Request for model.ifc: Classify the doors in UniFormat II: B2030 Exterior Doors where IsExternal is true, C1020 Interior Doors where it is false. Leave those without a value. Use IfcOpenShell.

First a look at what the model holds.

```python
import ifcopenshell
import ifcopenshell.util.element

model = ifcopenshell.open("model.ifc")
print(model.schema)
print("classifications:", [c.Name for c in model.by_type("IfcClassification")])
values = [ifcopenshell.util.element.get_pset(e, "Pset_DoorCommon", "IsExternal") for e in model.by_type("IfcDoor")]
for value in (True, False, None):
    print("IsExternal", value, values.count(value))
```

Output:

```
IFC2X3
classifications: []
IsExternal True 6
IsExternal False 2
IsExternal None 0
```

```python
import ifcopenshell
import ifcopenshell.api.classification
import ifcopenshell.util.element

model = ifcopenshell.open("model.ifc")

# IFC2X3 requires Source and Edition and has no link from the project to the system.
system = model.create_entity("IfcClassification", Source="ASTM", Edition="E1557", Name="UniFormat II")

doors = model.by_type("IfcDoor")
external = {e: ifcopenshell.util.element.get_pset(e, "Pset_DoorCommon", "IsExternal") for e in doors}
for flag, code, name in ((True, "B2030", "Exterior Doors"), (False, "C1020", "Interior Doors")):
    products = [e for e in doors if external[e] is flag]
    ifcopenshell.api.classification.add_reference(
        model, products=products, classification=system, identification=code, name=name
    )
    print(code, len(products))

model.write("model_v2.ifc")
```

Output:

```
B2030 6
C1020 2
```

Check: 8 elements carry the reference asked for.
